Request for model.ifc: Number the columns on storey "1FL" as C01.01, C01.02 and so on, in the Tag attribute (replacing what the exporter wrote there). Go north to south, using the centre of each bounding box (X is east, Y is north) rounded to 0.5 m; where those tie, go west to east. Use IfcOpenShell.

First a look at what the model holds.

```python
import ifcopenshell
import ifcopenshell.util.element
import ifcopenshell.util.placement

model = ifcopenshell.open("model.ifc")
print(model.schema)
storey = next(s for s in model.by_type("IfcBuildingStorey") if s.Name == "1FL")
columns = [e for e in ifcopenshell.util.element.get_decomposition(storey) if e.is_a("IfcColumn")]
for e in sorted(columns, key=lambda e: e.id()):
    origin = ifcopenshell.util.placement.get_local_placement(e.ObjectPlacement)[:3, 3]
    print(e.id(), e.Tag, e.Name, origin.round(2) + 0.0, sep=" | ")
```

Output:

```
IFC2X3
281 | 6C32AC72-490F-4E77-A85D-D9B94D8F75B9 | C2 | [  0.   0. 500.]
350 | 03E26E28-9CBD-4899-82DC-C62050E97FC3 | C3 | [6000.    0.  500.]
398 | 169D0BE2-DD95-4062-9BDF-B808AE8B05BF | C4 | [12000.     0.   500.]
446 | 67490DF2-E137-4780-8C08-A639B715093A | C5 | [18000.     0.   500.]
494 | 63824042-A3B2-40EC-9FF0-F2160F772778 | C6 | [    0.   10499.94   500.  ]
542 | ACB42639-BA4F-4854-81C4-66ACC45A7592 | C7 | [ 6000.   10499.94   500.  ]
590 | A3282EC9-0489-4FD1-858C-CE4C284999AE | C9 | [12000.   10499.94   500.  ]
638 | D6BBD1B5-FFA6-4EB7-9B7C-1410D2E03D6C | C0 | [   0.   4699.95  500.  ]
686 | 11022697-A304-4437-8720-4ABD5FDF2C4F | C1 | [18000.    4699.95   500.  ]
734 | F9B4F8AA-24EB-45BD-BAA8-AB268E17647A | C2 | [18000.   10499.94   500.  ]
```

```python
import ifcopenshell
import ifcopenshell.geom
import ifcopenshell.util.element
import ifcopenshell.util.shape

model = ifcopenshell.open("model.ifc")
settings = ifcopenshell.geom.settings()
settings.set("use-world-coords", True)


def centre(element):
    shape = ifcopenshell.geom.create_shape(settings, element)
    return ifcopenshell.util.shape.get_bbox_centroid(shape.geometry)


storey = next(s for s in model.by_type("IfcBuildingStorey") if s.Name == "1FL")
columns = [e for e in ifcopenshell.util.element.get_decomposition(storey) if e.is_a("IfcColumn")]

# Insertion points can sit at a corner or the storey origin, so sort by the geometry (in metres).
centres = {e: centre(e) for e in columns}
columns.sort(key=lambda e: (-round(centres[e][1] / 0.5), centres[e][0]))

for i, e in enumerate(columns, start=1):
    number = f"C01.{i:02d}"
    e.Tag = number
    print(e.id(), number)

model.write("model_rev.ifc")
```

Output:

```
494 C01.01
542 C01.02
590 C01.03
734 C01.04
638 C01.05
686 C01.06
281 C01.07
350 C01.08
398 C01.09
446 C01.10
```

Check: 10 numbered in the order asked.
